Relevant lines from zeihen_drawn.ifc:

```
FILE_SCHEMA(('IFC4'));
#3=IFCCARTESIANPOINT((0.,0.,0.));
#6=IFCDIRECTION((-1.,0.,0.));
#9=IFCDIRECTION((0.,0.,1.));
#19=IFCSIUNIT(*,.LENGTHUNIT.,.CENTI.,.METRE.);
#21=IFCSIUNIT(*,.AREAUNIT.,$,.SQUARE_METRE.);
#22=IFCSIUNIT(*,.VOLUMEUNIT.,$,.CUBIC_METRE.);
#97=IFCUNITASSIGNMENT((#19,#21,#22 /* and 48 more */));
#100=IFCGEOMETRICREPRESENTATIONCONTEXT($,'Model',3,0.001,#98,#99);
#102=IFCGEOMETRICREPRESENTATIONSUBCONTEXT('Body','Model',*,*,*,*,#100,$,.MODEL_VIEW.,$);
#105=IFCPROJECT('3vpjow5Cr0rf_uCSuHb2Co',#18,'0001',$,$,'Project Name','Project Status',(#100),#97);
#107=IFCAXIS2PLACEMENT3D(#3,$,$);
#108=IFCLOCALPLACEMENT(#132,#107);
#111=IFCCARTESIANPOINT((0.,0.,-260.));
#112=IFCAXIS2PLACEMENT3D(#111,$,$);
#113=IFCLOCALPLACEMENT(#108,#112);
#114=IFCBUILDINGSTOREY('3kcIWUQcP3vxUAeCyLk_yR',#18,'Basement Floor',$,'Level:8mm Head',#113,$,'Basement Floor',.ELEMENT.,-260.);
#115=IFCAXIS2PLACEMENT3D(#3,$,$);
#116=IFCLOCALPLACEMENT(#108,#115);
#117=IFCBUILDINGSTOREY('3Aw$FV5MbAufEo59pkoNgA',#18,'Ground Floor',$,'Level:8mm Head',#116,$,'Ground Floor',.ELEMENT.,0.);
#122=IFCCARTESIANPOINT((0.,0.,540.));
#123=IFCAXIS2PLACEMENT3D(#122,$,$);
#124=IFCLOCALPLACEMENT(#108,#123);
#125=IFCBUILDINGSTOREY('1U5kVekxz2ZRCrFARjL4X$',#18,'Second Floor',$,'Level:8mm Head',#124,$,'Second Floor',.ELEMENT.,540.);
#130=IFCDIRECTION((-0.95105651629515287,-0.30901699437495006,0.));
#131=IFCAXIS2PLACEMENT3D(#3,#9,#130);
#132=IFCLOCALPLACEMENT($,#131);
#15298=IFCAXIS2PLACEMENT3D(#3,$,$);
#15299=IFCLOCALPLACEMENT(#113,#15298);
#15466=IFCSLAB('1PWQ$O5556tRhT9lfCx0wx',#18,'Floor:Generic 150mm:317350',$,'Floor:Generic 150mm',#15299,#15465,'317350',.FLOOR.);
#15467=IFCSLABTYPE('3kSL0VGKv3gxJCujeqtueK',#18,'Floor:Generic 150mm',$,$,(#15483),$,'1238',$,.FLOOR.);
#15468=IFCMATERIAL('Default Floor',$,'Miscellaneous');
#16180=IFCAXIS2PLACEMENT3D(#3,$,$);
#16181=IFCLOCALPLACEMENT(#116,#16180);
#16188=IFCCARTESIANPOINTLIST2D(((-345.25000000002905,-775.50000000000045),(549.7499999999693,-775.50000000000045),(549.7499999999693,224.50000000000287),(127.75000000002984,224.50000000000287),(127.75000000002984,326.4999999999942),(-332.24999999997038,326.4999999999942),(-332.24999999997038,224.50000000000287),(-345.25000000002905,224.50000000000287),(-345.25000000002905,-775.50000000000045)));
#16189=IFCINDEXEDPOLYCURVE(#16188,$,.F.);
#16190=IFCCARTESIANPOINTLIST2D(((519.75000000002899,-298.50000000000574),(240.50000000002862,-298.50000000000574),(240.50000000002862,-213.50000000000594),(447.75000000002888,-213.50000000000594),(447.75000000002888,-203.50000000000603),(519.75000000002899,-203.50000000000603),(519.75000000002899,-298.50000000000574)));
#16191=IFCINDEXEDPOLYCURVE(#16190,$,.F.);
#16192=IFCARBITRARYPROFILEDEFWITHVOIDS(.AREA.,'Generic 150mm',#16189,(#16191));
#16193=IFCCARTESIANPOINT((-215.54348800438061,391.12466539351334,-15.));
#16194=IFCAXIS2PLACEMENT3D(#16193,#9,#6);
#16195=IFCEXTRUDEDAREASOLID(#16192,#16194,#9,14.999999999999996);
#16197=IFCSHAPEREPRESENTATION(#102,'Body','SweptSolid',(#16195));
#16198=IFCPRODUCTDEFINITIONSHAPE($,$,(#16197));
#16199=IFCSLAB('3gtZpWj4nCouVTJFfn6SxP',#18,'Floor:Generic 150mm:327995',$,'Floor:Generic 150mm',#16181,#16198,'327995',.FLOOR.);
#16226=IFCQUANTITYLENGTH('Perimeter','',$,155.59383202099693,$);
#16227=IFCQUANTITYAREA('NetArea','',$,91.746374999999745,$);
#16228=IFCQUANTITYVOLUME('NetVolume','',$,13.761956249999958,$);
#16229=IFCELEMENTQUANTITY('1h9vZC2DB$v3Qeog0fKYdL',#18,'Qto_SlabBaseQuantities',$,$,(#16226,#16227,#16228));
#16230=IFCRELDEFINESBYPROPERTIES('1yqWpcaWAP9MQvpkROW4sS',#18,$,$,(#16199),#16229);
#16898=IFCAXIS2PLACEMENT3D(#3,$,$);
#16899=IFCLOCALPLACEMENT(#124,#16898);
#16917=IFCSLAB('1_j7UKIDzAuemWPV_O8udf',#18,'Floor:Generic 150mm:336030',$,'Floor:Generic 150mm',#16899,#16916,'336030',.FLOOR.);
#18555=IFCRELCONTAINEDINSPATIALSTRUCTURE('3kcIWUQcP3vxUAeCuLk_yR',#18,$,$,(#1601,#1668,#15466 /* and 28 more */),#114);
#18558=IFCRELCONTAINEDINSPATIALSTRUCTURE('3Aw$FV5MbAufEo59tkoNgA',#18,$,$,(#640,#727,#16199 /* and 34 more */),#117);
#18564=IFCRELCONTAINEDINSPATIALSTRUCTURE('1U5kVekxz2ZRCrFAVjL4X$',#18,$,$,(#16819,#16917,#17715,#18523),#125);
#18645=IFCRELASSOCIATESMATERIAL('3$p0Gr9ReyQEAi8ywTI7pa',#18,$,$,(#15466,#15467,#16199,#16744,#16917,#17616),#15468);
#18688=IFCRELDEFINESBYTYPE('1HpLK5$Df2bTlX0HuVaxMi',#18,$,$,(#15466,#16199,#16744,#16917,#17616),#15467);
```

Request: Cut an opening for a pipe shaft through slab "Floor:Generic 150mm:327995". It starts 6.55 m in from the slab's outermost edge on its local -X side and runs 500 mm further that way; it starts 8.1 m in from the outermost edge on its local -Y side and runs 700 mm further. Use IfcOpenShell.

```python
import numpy as np
import ifcopenshell
import ifcopenshell.api.feature
import ifcopenshell.api.geometry
import ifcopenshell.api.pset
import ifcopenshell.api.root
import ifcopenshell.geom
import ifcopenshell.util.element
import ifcopenshell.util.placement
import ifcopenshell.util.representation
import ifcopenshell.util.shape
import ifcopenshell.util.unit

model = ifcopenshell.open("zeihen_drawn.ifc")
unit_scale = ifcopenshell.util.unit.calculate_unit_scale(model)
area_scale = ifcopenshell.util.unit.calculate_unit_scale(model, "AREAUNIT")
volume_scale = ifcopenshell.util.unit.calculate_unit_scale(model, "VOLUMEUNIT")
settings = ifcopenshell.geom.settings()


def volume(element):
    """Net volume in cubic metres, openings subtracted."""
    shape = ifcopenshell.geom.create_shape(settings, element)
    return ifcopenshell.util.shape.get_volume(shape.geometry)


slab = model.by_id(16199)
before = volume(slab)

# Extent in the slab's own axes, in metres. The edges named are its -X and -Y sides.
slab_shape = ifcopenshell.geom.create_shape(settings, slab)
vertices = ifcopenshell.util.shape.get_vertices(slab_shape.geometry)
x_min, y_min, bottom = vertices.min(axis=0)
top = vertices[:, 2].max()

opening = ifcopenshell.api.root.create_entity(model, ifc_class="IfcOpeningElement", name="Pipe shaft opening", predefined_type="OPENING")
context = ifcopenshell.util.representation.get_context(model, "Model", "Body", "MODEL_VIEW")
width, depth = 0.5, 0.7
outline = [(0.0, 0.0), (width, 0.0), (width, depth), (0.0, depth), (0.0, 0.0)]
# Overshoot both faces by 50 mm so the cut is clean.
shape = ifcopenshell.api.geometry.add_slab_representation(
    model, context=context, depth=top - bottom + 0.1, polyline=outline
)
ifcopenshell.api.geometry.assign_representation(model, product=opening, representation=shape)

matrix = ifcopenshell.util.placement.get_local_placement(slab.ObjectPlacement)
matrix[:, 3] = matrix @ np.append(np.array([x_min + 6.55, y_min + 8.1, bottom - 0.05]) / unit_scale, 1.0)
ifcopenshell.api.geometry.edit_object_placement(model, product=opening, matrix=matrix, is_si=False)
ifcopenshell.api.feature.add_feature(model, feature=opening, element=slab)

after = volume(slab)

# Update the slab's stored quantities.
qto = model.by_id(ifcopenshell.util.element.get_pset(slab, "Qto_SlabBaseQuantities", should_inherit=False)["id"])
ifcopenshell.api.pset.edit_qto(model, qto=qto, properties={
    "NetArea": after / (top - bottom) / area_scale,
    "NetVolume": after / volume_scale,
})

print(f"slab volume {before:.3f} -> {after:.3f} m3")

model.write("zeihen_drawn-out.ifc")
```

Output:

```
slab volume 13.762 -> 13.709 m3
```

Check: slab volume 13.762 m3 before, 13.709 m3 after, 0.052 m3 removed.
